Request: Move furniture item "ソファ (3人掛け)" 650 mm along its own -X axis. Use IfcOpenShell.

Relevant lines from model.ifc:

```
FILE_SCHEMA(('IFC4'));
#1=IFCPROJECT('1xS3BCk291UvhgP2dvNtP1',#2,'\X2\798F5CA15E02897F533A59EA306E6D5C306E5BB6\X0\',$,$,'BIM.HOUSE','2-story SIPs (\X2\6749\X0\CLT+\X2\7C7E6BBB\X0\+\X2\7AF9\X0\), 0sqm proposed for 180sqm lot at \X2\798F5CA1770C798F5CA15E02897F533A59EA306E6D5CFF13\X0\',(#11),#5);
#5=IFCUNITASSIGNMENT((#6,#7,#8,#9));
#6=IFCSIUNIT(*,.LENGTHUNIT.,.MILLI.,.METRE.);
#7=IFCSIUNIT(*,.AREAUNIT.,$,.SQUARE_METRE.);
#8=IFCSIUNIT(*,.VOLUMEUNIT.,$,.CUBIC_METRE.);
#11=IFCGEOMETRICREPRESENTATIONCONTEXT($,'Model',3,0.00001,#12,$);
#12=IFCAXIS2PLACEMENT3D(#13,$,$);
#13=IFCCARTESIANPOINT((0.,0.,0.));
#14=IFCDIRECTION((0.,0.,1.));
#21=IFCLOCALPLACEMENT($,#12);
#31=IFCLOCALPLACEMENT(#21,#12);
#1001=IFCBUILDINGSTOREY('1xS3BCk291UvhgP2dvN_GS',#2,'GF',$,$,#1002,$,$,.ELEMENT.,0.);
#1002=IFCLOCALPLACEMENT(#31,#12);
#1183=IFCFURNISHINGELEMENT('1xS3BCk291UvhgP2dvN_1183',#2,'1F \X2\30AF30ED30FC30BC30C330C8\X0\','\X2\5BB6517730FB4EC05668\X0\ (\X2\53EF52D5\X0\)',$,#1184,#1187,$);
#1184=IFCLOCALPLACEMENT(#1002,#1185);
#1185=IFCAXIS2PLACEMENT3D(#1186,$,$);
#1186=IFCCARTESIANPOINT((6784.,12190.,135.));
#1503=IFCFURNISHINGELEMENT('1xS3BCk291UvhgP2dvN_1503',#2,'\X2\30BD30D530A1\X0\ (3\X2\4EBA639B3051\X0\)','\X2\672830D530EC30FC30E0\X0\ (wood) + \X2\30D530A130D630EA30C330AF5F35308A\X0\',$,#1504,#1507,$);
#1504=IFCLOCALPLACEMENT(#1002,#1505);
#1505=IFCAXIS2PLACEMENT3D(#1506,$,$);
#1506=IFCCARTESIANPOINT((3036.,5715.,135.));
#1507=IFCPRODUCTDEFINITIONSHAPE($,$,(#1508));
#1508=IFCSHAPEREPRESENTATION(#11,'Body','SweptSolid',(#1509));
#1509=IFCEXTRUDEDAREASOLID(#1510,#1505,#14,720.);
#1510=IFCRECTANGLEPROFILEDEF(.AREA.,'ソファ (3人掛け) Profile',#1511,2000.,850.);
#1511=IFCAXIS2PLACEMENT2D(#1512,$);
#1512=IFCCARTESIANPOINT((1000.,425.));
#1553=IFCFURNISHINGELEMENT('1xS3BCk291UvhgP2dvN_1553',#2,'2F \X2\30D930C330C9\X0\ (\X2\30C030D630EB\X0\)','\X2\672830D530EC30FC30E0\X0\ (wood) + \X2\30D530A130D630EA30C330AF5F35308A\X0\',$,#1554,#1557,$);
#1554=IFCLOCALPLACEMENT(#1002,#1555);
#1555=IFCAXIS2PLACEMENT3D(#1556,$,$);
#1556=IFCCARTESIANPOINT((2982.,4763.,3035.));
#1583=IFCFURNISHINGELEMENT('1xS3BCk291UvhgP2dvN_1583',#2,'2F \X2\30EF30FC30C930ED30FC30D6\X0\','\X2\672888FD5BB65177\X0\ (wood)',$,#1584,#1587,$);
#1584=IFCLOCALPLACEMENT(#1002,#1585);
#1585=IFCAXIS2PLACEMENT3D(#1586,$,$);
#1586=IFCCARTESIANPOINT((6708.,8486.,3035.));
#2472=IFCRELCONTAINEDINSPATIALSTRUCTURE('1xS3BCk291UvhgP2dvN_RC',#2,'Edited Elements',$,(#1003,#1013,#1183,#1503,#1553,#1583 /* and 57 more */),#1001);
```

```python
import ifcopenshell
import ifcopenshell.api.geometry
import ifcopenshell.util.placement
import ifcopenshell.util.unit

model = ifcopenshell.open("model.ifc")
unit_scale = ifcopenshell.util.unit.calculate_unit_scale(model)

item = model.by_guid("1xS3BCk291UvhgP2dvN_1503")
matrix = ifcopenshell.util.placement.get_local_placement(item.ObjectPlacement)
matrix[:3, 3] -= matrix[:3, 0] * 0.65 / unit_scale
ifcopenshell.api.geometry.edit_object_placement(model, product=item, matrix=matrix, is_si=False)

print(ifcopenshell.util.placement.get_local_placement(item.ObjectPlacement).round(3) + 0.0)

model.write("model_edited.ifc")
```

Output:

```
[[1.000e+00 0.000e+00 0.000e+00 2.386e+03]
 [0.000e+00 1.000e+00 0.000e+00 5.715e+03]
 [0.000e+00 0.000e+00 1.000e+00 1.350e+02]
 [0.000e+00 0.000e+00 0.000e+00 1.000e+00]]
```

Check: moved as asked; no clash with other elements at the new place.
